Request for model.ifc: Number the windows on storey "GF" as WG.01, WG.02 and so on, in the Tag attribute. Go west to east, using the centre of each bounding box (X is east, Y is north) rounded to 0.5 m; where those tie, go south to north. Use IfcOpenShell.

First a look at what the model holds.

```python
import ifcopenshell
import ifcopenshell.util.element
import ifcopenshell.util.placement

model = ifcopenshell.open("model.ifc")
print(model.schema)
storey = next(s for s in model.by_type("IfcBuildingStorey") if s.Name == "GF")
windows = [e for e in ifcopenshell.util.element.get_decomposition(storey) if e.is_a("IfcWindow")]
for e in sorted(windows, key=lambda e: e.id()):
    origin = ifcopenshell.util.placement.get_local_placement(e.ObjectPlacement)[:3, 3]
    print(e.id(), e.Tag, e.Name, origin.round(2) + 0.0, sep=" | ")
```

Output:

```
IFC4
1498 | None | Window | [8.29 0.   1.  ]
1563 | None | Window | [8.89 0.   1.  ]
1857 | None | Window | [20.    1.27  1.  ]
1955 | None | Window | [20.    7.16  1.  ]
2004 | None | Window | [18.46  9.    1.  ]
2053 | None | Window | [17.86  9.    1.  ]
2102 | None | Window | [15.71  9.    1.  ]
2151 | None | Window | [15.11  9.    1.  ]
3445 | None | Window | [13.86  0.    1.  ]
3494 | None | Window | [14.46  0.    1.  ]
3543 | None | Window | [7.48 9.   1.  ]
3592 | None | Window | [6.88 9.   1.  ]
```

```python
import ifcopenshell
import ifcopenshell.geom
import ifcopenshell.util.element
import ifcopenshell.util.shape

model = ifcopenshell.open("model.ifc")
settings = ifcopenshell.geom.settings()
settings.set("use-world-coords", True)


def centre(element):
    shape = ifcopenshell.geom.create_shape(settings, element)
    return ifcopenshell.util.shape.get_bbox_centroid(shape.geometry)


storey = next(s for s in model.by_type("IfcBuildingStorey") if s.Name == "GF")
windows = [e for e in ifcopenshell.util.element.get_decomposition(storey) if e.is_a("IfcWindow")]

# Insertion points can sit at a corner or the storey origin, so sort by the geometry (in metres).
centres = {e: centre(e) for e in windows}
windows.sort(key=lambda e: (round(centres[e][0] / 0.5), centres[e][1]))

for i, e in enumerate(windows, start=1):
    number = f"WG.{i:02d}"
    e.Tag = number
    print(e.id(), number)

model.write("model_v2.ifc")
```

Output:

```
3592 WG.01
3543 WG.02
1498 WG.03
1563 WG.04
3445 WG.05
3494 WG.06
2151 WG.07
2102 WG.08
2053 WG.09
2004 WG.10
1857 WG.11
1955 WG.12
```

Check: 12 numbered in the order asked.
